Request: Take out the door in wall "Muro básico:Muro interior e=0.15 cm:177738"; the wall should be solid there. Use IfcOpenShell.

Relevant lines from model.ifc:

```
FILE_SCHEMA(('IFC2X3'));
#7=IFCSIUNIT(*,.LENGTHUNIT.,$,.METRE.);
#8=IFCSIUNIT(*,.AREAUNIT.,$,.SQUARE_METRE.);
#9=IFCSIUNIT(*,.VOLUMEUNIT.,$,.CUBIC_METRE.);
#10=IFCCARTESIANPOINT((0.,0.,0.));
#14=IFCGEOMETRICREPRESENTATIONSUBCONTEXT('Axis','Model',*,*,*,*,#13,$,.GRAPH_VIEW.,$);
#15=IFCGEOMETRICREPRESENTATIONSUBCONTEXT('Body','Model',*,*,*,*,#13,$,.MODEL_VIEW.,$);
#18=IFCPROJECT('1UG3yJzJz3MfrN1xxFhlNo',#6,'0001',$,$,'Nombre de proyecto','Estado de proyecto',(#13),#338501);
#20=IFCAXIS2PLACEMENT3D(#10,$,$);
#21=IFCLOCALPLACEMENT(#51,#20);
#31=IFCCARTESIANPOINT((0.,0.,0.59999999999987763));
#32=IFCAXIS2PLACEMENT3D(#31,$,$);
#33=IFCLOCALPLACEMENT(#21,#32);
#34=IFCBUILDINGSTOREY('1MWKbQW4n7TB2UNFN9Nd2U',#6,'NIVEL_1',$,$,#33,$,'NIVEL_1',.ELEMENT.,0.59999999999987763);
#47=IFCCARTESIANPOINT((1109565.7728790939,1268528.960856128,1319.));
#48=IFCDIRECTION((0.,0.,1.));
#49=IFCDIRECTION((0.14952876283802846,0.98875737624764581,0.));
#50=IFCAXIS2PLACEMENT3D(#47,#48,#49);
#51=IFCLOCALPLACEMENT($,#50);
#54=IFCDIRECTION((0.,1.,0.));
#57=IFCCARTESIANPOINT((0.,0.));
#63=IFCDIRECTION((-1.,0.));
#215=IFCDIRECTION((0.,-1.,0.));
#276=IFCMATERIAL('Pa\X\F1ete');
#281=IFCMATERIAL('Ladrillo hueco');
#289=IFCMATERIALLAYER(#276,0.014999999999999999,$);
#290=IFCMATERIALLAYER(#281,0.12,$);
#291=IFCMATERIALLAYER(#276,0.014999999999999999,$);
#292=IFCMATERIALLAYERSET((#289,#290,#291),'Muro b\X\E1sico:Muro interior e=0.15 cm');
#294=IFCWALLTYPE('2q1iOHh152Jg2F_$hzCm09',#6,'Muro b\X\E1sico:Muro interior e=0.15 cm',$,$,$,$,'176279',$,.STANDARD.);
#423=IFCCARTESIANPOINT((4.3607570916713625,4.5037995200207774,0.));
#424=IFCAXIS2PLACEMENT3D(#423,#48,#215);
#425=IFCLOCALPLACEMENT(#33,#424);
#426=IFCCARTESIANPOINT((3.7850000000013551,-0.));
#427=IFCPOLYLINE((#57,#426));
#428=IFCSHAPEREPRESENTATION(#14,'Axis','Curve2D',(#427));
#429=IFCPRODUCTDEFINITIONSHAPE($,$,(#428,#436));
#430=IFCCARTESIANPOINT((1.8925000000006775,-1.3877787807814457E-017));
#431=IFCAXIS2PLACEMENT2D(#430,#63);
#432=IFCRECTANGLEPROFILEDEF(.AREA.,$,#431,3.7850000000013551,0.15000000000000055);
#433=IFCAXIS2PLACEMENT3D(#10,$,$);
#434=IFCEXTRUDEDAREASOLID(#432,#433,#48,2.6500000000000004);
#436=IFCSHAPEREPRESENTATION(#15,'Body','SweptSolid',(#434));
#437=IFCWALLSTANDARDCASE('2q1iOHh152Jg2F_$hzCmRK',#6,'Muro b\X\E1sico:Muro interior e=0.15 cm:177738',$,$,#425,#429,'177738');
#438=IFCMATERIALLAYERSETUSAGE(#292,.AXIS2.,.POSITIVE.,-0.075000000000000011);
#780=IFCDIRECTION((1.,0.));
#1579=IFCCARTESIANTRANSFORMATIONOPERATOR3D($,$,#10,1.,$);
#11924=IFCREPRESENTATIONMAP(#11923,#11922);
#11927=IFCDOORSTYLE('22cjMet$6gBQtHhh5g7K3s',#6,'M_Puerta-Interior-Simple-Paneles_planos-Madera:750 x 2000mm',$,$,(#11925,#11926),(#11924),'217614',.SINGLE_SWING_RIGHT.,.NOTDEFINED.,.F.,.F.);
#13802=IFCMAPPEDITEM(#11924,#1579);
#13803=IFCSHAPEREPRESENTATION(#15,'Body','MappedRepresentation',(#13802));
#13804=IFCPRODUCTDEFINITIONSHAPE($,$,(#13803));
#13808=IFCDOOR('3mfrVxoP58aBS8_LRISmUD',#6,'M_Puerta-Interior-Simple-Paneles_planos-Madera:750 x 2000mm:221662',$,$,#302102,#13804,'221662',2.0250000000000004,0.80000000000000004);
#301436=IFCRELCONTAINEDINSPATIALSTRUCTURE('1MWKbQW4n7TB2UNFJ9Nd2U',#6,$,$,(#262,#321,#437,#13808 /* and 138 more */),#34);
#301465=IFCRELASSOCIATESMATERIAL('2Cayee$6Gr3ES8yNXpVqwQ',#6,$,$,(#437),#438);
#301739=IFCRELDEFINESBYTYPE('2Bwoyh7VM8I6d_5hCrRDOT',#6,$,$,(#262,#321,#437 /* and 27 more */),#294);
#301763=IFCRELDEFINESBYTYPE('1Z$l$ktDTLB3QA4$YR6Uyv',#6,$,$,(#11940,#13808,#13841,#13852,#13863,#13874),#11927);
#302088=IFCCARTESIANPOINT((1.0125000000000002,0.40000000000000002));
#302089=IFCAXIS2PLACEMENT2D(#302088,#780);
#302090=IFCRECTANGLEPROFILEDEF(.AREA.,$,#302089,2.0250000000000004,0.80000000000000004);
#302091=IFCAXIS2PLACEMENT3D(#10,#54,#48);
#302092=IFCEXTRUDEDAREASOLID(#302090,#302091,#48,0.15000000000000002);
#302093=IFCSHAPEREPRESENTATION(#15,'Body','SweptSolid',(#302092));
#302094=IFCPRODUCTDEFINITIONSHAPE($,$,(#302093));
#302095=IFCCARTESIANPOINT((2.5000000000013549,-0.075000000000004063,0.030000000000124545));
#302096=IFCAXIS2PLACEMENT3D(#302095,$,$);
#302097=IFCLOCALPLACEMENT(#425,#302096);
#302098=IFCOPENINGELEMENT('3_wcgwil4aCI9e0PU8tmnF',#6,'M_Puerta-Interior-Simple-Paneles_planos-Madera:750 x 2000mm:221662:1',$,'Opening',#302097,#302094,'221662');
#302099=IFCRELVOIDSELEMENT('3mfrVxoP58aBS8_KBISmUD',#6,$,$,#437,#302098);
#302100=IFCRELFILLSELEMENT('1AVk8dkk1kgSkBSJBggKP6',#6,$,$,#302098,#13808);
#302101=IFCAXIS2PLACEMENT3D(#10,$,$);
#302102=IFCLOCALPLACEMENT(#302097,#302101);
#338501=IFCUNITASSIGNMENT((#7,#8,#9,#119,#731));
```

```python
import ifcopenshell
import ifcopenshell.api.feature
import ifcopenshell.api.root
import ifcopenshell.geom
import ifcopenshell.util.shape

model = ifcopenshell.open("model.ifc")
settings = ifcopenshell.geom.settings()


def volume(element):
    """Net volume in cubic metres, openings subtracted."""
    shape = ifcopenshell.geom.create_shape(settings, element)
    return ifcopenshell.util.shape.get_volume(shape.geometry)


door = model.by_guid("3mfrVxoP58aBS8_LRISmUD")
opening = door.FillsVoids[0].RelatingOpeningElement
wall = opening.VoidsElements[0].RelatingBuildingElement
before = volume(wall)

ifcopenshell.api.root.remove_product(model, product=door)
ifcopenshell.api.feature.remove_feature(model, feature=opening)

after = volume(wall)

print(f"wall volume {before:.3f} -> {after:.3f} m3")

model.write("model_rev.ifc")
```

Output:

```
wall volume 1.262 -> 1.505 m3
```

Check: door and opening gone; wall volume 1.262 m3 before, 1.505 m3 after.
